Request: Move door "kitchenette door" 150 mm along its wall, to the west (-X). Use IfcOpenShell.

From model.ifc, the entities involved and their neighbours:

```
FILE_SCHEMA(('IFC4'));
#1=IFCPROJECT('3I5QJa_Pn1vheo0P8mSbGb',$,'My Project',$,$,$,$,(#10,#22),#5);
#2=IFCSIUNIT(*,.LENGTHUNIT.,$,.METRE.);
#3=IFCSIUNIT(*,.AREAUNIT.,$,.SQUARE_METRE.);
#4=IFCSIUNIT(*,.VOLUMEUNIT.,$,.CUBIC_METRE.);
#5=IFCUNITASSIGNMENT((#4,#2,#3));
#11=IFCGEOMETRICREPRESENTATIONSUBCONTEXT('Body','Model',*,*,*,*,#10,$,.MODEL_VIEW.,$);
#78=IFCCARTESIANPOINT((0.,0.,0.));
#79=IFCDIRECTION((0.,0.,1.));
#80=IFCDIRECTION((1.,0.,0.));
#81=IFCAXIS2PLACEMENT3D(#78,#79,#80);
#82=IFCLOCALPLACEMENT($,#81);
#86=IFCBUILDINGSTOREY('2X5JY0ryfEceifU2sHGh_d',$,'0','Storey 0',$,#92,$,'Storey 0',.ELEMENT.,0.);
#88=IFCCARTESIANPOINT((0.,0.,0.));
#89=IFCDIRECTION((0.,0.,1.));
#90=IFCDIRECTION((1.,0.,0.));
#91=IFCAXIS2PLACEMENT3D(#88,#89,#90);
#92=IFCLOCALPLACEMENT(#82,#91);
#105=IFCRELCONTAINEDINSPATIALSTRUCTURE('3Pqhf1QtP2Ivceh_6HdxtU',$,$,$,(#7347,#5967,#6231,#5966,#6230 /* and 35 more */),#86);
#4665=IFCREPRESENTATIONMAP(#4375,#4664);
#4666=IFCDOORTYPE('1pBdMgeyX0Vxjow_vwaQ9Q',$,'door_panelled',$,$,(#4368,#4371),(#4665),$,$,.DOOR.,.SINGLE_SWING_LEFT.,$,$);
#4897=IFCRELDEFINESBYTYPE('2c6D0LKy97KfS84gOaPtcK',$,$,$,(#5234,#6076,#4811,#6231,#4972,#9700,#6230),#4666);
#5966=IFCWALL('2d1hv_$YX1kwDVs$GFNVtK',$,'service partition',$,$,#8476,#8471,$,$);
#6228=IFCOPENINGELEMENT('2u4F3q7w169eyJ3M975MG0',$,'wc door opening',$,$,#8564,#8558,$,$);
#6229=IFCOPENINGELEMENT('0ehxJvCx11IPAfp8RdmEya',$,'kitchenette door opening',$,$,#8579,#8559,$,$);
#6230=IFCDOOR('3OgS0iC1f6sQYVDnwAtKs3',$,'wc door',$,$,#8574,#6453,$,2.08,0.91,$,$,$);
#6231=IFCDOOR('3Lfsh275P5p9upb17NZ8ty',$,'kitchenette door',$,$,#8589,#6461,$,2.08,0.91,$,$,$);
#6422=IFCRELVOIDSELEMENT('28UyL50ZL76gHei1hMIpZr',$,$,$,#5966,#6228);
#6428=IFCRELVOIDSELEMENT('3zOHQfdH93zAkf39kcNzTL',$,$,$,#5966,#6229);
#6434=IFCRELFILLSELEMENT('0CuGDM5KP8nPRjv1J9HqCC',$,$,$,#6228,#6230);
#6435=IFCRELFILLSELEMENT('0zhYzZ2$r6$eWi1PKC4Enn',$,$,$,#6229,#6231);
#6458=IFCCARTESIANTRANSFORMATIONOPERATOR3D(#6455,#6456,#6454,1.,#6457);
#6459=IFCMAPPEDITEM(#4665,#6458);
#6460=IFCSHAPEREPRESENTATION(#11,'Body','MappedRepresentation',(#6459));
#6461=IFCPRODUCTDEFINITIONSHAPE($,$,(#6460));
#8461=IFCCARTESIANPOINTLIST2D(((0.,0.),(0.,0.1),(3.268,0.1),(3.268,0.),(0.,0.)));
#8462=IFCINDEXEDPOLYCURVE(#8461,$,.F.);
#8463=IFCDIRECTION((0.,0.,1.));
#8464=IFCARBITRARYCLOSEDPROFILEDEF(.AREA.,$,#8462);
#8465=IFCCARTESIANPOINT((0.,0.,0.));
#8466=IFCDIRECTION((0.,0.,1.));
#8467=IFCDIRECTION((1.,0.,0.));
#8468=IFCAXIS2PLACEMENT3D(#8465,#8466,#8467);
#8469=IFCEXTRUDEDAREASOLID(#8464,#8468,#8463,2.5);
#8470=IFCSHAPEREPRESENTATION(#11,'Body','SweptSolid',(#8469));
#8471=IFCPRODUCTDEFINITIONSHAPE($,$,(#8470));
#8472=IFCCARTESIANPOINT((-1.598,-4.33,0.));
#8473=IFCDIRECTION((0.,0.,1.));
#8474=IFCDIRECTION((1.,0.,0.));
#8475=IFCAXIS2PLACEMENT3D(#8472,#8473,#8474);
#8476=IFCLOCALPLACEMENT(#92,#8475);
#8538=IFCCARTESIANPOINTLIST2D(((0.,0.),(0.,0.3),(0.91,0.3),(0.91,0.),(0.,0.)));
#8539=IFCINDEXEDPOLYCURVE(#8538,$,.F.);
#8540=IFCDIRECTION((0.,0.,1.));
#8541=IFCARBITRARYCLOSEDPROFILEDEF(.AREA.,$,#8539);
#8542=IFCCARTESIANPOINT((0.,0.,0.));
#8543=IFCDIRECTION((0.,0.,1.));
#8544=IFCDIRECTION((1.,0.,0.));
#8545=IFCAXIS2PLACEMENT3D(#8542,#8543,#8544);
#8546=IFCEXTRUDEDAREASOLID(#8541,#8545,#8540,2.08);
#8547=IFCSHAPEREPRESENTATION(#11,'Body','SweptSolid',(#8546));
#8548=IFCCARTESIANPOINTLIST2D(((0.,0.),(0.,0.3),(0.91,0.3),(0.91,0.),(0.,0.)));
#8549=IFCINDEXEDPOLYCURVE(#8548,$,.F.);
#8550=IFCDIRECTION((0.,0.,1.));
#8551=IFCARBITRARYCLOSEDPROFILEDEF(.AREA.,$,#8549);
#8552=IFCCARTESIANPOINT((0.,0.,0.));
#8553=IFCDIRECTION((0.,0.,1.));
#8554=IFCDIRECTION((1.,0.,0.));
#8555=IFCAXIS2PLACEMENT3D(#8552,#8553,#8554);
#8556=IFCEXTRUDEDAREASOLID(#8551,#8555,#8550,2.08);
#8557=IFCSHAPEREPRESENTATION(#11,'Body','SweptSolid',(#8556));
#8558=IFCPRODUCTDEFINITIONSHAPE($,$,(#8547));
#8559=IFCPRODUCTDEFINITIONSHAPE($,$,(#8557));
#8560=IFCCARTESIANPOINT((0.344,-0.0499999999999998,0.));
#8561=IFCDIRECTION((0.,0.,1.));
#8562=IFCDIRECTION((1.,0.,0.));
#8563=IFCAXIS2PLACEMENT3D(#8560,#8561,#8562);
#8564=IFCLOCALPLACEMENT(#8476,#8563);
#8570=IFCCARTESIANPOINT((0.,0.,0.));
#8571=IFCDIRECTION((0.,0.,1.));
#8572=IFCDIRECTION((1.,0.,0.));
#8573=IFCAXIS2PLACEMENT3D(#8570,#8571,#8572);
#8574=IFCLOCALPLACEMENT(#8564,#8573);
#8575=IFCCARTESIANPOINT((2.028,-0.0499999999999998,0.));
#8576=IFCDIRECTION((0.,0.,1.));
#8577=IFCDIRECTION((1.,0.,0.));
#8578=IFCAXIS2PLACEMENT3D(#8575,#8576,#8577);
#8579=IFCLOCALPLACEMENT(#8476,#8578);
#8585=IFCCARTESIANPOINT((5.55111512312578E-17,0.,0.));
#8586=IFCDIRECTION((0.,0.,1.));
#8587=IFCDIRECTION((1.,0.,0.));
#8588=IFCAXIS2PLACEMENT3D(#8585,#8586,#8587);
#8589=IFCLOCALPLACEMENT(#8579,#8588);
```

```python
import ifcopenshell
import ifcopenshell.api.geometry
import ifcopenshell.util.placement
import ifcopenshell.util.unit

model = ifcopenshell.open("model.ifc")
unit_scale = ifcopenshell.util.unit.calculate_unit_scale(model)

door = model.by_guid("3Lfsh275P5p9upb17NZ8ty")
opening = door.FillsVoids[0].RelatingOpeningElement
wall = opening.VoidsElements[0].RelatingBuildingElement

wall_matrix = ifcopenshell.util.placement.get_local_placement(wall.ObjectPlacement)
shift = wall_matrix[:3, 0] * -0.15 / unit_scale
before = ifcopenshell.util.placement.get_local_placement(door.ObjectPlacement)[:3, 3].copy()

# The door is placed relative to its opening, so it follows when the opening moves.
matrix = ifcopenshell.util.placement.get_local_placement(opening.ObjectPlacement)
matrix[:3, 3] += shift
ifcopenshell.api.geometry.edit_object_placement(
    model, product=opening, matrix=matrix, is_si=False, should_transform_children=True
)

after = ifcopenshell.util.placement.get_local_placement(door.ObjectPlacement)[:3, 3]
print("door moved by", (after - before).round(3) + 0.0)

model.write("model_updated.ifc")
```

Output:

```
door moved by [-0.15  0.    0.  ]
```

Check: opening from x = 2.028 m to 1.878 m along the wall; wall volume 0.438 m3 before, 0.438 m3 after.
